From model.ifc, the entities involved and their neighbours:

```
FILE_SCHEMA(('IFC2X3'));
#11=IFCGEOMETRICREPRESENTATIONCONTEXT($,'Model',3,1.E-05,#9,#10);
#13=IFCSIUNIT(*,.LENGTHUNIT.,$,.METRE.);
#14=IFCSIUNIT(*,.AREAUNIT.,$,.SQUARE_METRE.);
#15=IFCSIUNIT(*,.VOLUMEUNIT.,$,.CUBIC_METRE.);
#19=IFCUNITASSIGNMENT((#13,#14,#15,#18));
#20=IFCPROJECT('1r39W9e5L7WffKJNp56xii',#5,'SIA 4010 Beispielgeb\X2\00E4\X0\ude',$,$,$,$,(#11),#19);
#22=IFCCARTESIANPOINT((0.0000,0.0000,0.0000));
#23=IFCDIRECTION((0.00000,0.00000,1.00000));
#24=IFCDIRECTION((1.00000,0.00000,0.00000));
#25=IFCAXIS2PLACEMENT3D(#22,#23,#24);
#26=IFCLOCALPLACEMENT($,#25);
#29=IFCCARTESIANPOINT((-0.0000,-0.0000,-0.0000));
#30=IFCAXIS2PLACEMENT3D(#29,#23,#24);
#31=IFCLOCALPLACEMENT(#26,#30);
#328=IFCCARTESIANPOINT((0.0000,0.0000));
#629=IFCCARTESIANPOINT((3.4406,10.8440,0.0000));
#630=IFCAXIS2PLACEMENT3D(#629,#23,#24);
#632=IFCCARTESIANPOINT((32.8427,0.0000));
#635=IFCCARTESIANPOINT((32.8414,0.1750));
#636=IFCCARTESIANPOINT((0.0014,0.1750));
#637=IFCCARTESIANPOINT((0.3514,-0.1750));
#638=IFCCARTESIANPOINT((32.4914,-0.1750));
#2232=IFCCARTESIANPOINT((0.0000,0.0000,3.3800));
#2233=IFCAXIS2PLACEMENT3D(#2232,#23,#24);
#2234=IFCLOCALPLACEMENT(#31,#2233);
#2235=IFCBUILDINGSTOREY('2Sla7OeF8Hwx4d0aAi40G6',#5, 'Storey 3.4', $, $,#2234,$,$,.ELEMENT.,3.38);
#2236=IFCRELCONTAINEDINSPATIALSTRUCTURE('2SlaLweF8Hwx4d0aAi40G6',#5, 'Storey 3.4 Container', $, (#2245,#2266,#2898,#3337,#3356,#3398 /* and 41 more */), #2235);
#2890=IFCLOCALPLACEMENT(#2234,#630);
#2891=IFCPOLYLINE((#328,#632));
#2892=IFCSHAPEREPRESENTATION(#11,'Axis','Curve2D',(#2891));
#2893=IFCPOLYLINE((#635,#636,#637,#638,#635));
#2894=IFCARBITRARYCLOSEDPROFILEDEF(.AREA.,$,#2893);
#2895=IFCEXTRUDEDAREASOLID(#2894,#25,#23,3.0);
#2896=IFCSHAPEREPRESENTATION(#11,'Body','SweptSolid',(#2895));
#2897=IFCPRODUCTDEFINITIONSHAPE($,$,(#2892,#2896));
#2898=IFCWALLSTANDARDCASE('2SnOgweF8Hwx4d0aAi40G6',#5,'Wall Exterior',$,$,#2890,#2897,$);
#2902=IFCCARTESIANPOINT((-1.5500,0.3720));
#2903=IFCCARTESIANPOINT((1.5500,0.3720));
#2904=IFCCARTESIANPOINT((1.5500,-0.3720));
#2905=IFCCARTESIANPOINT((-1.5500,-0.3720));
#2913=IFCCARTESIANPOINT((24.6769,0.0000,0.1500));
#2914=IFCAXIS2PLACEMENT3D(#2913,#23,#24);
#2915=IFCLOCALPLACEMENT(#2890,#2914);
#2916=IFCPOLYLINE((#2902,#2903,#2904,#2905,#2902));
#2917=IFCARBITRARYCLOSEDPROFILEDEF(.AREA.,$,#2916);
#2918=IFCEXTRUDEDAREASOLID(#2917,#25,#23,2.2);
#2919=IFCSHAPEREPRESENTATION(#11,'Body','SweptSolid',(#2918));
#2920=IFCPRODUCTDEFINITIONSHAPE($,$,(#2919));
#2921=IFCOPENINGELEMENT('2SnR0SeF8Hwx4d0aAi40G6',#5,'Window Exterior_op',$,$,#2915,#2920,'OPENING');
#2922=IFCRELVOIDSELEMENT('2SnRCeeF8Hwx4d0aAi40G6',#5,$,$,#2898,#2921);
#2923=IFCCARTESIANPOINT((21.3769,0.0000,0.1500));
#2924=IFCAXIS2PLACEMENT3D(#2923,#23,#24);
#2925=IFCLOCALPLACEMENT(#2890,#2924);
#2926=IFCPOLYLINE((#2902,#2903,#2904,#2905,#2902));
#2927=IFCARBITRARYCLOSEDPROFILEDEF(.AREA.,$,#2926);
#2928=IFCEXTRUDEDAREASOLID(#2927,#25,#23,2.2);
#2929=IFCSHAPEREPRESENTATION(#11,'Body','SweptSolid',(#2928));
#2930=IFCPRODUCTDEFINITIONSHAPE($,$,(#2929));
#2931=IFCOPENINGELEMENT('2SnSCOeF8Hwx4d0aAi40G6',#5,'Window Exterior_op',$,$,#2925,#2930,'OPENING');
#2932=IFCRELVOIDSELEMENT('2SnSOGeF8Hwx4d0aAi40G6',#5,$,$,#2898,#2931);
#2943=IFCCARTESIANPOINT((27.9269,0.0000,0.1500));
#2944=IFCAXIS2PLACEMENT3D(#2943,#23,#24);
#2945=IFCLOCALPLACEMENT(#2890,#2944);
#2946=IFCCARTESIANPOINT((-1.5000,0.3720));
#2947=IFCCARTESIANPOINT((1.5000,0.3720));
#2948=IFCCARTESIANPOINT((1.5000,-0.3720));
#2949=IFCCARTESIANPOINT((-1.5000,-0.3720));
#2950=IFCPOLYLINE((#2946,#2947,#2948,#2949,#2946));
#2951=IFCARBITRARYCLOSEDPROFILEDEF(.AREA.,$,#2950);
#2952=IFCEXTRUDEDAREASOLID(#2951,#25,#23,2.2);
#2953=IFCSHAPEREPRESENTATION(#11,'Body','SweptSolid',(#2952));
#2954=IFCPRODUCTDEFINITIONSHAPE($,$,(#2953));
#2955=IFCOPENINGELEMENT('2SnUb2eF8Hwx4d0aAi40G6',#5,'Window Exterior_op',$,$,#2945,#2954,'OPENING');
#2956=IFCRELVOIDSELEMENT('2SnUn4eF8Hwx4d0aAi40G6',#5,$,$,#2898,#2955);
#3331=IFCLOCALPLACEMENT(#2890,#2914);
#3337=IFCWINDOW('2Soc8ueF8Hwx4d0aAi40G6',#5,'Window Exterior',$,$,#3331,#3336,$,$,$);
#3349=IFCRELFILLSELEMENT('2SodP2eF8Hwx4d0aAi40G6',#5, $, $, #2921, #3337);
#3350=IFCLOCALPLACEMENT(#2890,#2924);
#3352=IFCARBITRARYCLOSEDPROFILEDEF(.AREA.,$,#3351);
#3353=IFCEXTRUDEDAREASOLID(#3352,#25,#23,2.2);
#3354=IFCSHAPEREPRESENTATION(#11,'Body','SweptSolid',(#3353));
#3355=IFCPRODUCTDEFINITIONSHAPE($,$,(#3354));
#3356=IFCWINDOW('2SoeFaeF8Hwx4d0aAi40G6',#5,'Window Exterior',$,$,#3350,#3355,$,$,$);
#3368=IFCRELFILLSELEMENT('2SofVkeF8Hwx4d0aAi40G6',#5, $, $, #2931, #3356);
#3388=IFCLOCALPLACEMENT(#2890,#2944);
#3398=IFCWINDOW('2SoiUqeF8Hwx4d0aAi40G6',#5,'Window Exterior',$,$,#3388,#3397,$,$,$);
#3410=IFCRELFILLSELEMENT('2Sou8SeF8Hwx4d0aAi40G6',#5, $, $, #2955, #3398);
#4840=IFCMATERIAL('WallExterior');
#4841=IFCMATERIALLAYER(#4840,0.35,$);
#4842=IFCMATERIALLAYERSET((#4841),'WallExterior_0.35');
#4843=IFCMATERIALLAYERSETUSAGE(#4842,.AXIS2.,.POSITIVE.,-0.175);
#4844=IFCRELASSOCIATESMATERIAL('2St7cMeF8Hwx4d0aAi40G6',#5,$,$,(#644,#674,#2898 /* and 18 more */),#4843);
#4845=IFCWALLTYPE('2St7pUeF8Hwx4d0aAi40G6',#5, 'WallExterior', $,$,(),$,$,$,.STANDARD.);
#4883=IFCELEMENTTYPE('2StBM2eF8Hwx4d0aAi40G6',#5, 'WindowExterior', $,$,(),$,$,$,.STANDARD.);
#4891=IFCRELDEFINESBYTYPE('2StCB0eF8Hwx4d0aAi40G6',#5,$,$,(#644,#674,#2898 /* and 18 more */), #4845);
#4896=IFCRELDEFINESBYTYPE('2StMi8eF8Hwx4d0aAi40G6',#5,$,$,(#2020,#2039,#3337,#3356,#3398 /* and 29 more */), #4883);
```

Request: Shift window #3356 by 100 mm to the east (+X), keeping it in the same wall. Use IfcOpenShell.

```python
import ifcopenshell
import ifcopenshell.api.geometry
import ifcopenshell.util.placement
import ifcopenshell.util.unit

model = ifcopenshell.open("model.ifc")
unit_scale = ifcopenshell.util.unit.calculate_unit_scale(model)

window = model.by_id(3356)
opening = window.FillsVoids[0].RelatingOpeningElement
wall = opening.VoidsElements[0].RelatingBuildingElement

wall_matrix = ifcopenshell.util.placement.get_local_placement(wall.ObjectPlacement)
shift = wall_matrix[:3, 0] * 0.1 / unit_scale
before = ifcopenshell.util.placement.get_local_placement(window.ObjectPlacement)[:3, 3].copy()

# The window is not placed relative to its opening, so move both.
for product in (opening, window):
    matrix = ifcopenshell.util.placement.get_local_placement(product.ObjectPlacement)
    matrix[:3, 3] += shift
    ifcopenshell.api.geometry.edit_object_placement(model, product=product, matrix=matrix, is_si=False)

after = ifcopenshell.util.placement.get_local_placement(window.ObjectPlacement)[:3, 3]
print("window moved by", (after - before).round(3) + 0.0)

model.write("model_edited.ifc")
```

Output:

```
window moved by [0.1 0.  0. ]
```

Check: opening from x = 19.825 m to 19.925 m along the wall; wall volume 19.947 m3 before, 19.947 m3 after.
